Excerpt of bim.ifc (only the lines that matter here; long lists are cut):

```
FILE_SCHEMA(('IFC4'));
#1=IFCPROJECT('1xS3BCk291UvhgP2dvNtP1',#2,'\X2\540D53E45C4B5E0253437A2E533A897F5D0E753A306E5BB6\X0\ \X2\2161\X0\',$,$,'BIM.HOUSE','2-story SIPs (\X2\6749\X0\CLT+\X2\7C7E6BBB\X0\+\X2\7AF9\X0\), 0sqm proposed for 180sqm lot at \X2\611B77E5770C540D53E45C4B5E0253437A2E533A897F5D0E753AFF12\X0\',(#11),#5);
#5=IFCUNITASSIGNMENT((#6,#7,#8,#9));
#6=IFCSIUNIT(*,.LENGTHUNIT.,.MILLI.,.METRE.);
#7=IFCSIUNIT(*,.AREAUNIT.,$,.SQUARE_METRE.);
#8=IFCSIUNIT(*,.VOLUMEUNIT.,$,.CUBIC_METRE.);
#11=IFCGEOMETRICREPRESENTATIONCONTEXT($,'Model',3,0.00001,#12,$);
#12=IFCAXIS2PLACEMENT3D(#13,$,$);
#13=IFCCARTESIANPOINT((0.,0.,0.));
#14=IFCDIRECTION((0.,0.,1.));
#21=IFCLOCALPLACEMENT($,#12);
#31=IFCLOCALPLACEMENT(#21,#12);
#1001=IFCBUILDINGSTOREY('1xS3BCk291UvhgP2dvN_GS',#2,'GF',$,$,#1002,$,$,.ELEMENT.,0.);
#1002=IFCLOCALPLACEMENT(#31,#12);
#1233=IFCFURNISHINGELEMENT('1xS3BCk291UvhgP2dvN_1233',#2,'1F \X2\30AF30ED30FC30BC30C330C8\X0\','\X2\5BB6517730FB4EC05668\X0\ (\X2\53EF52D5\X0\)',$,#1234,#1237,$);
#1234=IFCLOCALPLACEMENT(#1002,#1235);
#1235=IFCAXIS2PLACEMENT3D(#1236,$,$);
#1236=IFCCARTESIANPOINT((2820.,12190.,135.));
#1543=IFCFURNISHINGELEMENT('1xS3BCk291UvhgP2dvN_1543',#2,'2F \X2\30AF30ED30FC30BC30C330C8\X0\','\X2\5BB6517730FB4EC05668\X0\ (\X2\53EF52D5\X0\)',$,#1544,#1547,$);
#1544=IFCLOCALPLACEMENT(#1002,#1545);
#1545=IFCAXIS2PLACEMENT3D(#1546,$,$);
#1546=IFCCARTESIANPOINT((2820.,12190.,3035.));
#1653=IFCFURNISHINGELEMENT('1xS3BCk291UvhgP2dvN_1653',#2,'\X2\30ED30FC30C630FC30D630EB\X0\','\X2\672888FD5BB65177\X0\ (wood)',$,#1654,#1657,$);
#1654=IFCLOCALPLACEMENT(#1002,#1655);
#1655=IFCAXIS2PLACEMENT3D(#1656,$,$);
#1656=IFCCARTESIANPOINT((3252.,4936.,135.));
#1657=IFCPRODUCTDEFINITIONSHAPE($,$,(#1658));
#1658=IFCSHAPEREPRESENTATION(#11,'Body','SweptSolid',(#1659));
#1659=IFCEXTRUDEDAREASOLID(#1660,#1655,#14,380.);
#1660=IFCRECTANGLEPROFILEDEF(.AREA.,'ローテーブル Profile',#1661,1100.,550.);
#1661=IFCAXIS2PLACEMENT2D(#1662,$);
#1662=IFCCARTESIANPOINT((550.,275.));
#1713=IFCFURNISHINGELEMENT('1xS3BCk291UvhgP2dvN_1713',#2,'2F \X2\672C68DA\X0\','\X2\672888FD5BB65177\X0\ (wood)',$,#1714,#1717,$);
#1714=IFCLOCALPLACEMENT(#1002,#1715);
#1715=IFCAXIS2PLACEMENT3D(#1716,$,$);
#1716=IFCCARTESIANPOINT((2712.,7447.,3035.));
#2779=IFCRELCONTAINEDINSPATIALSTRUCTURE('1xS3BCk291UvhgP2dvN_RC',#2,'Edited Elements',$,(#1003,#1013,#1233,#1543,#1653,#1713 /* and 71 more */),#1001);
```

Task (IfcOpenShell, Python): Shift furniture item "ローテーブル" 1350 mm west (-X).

```python
import ifcopenshell
import ifcopenshell.api.geometry
import ifcopenshell.util.placement
import ifcopenshell.util.unit

model = ifcopenshell.open("bim.ifc")
unit_scale = ifcopenshell.util.unit.calculate_unit_scale(model)

item = model.by_id(1653)
matrix = ifcopenshell.util.placement.get_local_placement(item.ObjectPlacement)
matrix[0, 3] -= 1.35 / unit_scale
ifcopenshell.api.geometry.edit_object_placement(model, product=item, matrix=matrix, is_si=False)

print(ifcopenshell.util.placement.get_local_placement(item.ObjectPlacement).round(3) + 0.0)

model.write("bim_rev.ifc")
```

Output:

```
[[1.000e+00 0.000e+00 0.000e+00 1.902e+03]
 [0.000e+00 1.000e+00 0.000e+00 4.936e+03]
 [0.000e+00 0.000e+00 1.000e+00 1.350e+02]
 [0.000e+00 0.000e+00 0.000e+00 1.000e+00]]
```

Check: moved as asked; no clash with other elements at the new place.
